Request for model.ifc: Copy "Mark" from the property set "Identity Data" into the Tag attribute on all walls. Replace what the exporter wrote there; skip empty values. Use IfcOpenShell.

First a look at what the model holds.

```python
import ifcopenshell
import ifcopenshell.util.element

model = ifcopenshell.open("model.ifc")
print(model.schema)
walls = model.by_type("IfcWall")
print(len(walls), "walls")
for e in walls[:8]:
    source = ifcopenshell.util.element.get_pset(e, "Identity Data", "Mark")
    target = e.Tag
    print(e.id(), repr(source), repr(target), sep=" | ")
```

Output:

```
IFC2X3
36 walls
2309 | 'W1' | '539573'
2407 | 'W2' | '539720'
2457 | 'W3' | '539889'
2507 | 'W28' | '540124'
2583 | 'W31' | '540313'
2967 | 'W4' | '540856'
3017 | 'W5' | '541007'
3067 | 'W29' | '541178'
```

```python
import ifcopenshell
import ifcopenshell.util.element

model = ifcopenshell.open("model.ifc")

count = 0
for e in model.by_type("IfcWall"):
    value = ifcopenshell.util.element.get_pset(e, "Identity Data", "Mark")
    current = e.Tag
    if not value or not value.strip() or current == value:
        continue
    e.Tag = value
    count += 1

print(count, "walls updated")

model.write("model_v2.ifc")
```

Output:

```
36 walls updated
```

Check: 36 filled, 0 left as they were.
